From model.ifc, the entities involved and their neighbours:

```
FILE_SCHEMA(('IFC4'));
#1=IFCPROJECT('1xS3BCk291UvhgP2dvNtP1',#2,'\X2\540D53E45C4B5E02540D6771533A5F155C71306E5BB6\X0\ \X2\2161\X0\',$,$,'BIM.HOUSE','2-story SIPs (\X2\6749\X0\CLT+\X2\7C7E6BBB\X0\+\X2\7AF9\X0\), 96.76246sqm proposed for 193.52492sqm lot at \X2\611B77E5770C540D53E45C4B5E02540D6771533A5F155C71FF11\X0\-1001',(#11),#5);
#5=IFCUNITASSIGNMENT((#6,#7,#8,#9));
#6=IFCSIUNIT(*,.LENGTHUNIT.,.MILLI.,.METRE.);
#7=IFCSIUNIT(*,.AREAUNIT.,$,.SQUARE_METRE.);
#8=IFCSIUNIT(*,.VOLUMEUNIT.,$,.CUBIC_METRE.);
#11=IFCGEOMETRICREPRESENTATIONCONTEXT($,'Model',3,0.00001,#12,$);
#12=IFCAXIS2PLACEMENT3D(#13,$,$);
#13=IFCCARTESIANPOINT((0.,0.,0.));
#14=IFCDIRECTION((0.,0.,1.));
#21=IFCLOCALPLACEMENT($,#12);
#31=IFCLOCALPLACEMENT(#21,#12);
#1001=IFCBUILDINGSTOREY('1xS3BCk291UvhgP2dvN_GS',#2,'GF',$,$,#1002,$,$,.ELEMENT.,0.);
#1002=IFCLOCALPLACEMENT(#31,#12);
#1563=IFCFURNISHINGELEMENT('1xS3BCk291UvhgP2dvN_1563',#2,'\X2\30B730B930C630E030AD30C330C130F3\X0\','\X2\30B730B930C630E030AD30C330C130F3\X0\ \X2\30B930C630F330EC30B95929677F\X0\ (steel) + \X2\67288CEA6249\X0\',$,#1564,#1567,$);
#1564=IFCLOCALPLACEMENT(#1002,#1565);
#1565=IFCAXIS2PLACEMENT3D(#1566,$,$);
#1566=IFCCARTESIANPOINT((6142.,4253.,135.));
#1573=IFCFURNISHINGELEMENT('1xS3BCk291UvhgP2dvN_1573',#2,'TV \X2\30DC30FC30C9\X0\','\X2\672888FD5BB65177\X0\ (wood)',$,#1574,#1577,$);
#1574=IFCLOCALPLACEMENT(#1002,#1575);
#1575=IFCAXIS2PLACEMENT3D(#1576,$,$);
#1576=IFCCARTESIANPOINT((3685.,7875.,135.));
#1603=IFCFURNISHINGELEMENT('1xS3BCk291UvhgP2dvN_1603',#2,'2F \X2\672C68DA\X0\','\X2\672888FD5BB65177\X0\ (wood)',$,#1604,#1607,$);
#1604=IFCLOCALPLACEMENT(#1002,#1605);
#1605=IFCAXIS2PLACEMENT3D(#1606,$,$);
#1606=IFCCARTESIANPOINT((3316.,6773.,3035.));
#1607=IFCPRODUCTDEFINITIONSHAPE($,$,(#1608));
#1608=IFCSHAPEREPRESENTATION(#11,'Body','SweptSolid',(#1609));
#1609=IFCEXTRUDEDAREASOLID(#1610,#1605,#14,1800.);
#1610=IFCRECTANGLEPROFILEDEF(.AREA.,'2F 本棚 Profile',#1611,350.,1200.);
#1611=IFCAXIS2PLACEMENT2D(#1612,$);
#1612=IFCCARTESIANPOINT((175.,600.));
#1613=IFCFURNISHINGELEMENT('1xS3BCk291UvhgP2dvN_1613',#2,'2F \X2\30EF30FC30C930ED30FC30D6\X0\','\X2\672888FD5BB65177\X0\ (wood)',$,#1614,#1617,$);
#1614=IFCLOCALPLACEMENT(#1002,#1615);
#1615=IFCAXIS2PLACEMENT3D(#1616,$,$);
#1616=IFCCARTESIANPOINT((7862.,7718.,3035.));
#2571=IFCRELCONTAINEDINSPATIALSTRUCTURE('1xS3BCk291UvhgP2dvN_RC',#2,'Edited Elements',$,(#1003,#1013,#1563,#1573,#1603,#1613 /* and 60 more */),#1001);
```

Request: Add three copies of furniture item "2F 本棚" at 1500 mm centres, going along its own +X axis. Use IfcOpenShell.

```python
import ifcopenshell
import ifcopenshell.api.geometry
import ifcopenshell.api.root
import ifcopenshell.util.element
import ifcopenshell.util.placement
import ifcopenshell.util.unit

model = ifcopenshell.open("model.ifc")
unit_scale = ifcopenshell.util.unit.calculate_unit_scale(model)


def reuse_history(source, copy):
    """copy_class also copies each property set's owner history, people and application; keep the originals."""
    for rel in copy.IsDefinedBy:
        if rel.is_a("IfcRelDefinesByProperties") and (history := rel.RelatingPropertyDefinition.OwnerHistory):
            rel.RelatingPropertyDefinition.OwnerHistory = source.OwnerHistory
            ifcopenshell.util.element.remove_deep2(model, history)


source = model.by_guid("1xS3BCk291UvhgP2dvN_1603")
base = ifcopenshell.util.placement.get_local_placement(source.ObjectPlacement)
step = base[:3, 0] * 1.5 / unit_scale

for i in range(1, 4):
    copy = ifcopenshell.api.root.copy_class(model, product=source)
    copy.Representation = ifcopenshell.util.element.copy_deep(
        model, source.Representation, exclude=["IfcGeometricRepresentationContext", "IfcRepresentationMap"]
    )
    reuse_history(source, copy)
    matrix = base.copy()
    matrix[:3, 3] += i * step
    print("added at", matrix[:3, 3].round(3) + 0.0)
    ifcopenshell.api.geometry.edit_object_placement(model, product=copy, matrix=matrix, is_si=False)

model.write("model_updated.ifc")
```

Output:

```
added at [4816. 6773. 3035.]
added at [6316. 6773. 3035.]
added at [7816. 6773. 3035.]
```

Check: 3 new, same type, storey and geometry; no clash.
